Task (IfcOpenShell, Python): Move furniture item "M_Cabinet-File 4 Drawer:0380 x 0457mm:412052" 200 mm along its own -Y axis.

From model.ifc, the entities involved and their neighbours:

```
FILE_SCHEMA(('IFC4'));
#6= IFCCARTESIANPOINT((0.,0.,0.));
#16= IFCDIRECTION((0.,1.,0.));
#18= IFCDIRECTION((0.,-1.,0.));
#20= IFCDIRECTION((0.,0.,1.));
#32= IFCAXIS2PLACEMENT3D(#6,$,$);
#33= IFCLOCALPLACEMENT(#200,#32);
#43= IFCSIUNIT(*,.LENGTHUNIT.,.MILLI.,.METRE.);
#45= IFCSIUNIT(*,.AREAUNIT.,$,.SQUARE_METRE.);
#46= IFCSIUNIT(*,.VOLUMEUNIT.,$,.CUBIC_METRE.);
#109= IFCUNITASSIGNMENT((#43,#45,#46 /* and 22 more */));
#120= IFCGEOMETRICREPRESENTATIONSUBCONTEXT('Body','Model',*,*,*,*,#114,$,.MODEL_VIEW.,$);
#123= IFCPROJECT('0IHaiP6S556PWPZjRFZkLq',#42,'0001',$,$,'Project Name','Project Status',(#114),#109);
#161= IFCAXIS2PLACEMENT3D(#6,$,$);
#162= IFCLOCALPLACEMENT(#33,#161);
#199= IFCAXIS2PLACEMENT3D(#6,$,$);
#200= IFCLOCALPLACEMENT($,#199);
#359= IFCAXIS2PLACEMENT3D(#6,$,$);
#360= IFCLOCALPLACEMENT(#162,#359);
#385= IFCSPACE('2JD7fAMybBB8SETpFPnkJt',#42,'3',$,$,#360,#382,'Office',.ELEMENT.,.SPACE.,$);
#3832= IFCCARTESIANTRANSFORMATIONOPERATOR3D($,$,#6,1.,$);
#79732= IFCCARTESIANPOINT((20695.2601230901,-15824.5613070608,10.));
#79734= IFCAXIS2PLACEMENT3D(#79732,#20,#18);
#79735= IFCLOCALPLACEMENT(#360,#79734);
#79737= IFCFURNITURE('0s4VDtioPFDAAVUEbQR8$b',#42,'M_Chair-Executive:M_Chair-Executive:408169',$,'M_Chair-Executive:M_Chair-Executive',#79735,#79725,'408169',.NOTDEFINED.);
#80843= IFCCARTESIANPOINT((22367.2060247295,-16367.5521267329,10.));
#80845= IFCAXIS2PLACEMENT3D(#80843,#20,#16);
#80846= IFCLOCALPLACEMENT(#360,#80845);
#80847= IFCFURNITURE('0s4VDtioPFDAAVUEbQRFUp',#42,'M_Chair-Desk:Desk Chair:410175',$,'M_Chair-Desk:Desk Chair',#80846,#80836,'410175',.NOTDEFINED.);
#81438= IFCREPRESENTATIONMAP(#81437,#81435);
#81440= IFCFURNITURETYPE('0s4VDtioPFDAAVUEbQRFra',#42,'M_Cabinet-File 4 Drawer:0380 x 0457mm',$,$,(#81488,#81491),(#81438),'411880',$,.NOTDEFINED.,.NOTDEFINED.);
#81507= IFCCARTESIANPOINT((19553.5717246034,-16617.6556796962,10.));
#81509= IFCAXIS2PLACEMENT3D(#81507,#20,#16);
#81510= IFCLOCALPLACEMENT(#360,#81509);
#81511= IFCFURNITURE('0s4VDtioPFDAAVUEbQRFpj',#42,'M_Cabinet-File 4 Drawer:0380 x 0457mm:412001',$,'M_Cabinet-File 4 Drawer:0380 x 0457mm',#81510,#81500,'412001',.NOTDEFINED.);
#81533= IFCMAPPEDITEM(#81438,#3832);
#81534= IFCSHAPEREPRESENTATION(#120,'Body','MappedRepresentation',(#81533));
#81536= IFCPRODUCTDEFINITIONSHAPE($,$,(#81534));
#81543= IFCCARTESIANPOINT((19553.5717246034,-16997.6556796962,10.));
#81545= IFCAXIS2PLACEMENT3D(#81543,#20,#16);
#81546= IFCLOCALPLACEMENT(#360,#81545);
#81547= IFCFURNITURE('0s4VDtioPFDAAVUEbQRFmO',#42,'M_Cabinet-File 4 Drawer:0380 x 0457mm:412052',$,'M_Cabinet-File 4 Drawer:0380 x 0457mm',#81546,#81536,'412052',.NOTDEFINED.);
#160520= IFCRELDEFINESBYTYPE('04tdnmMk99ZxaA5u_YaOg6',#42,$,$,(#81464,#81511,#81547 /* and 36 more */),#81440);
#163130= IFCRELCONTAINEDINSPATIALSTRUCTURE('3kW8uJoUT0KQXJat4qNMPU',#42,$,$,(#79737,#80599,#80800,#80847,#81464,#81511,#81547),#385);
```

```python
import ifcopenshell
import ifcopenshell.api.geometry
import ifcopenshell.util.placement
import ifcopenshell.util.unit

model = ifcopenshell.open("model.ifc")
unit_scale = ifcopenshell.util.unit.calculate_unit_scale(model)

item = model.by_guid("0s4VDtioPFDAAVUEbQRFmO")
matrix = ifcopenshell.util.placement.get_local_placement(item.ObjectPlacement)
matrix[:3, 3] -= matrix[:3, 1] * 0.2 / unit_scale
ifcopenshell.api.geometry.edit_object_placement(model, product=item, matrix=matrix, is_si=False)

print(ifcopenshell.util.placement.get_local_placement(item.ObjectPlacement).round(3) + 0.0)

model.write("model_updated.ifc")
```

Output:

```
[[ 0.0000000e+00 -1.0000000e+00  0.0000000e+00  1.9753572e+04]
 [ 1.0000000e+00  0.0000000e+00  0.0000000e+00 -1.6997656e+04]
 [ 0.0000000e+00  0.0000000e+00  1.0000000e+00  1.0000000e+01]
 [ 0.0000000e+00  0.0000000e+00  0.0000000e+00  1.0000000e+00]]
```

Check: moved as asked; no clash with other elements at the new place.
